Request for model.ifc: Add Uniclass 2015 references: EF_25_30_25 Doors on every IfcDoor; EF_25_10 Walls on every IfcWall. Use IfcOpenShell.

First a look at what the model holds.

```python
import ifcopenshell

model = ifcopenshell.open("model.ifc")
print(model.schema)
print("classifications:", [c.Name for c in model.by_type("IfcClassification")])
for ifc_class in ("IfcDoor", "IfcRoof", "IfcStair", "IfcWall", "IfcWindow"):
    print(ifc_class, len(model.by_type(ifc_class)))
```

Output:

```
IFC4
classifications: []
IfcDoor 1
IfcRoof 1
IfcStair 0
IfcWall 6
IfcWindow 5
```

```python
import ifcopenshell
import ifcopenshell.api.classification

model = ifcopenshell.open("model.ifc")

system = ifcopenshell.api.classification.add_classification(model, classification="Uniclass 2015")

codes = {
    "IfcDoor": ("EF_25_30_25", "Doors"),
    "IfcWall": ("EF_25_10", "Walls"),
}
for ifc_class, (code, name) in codes.items():
    products = model.by_type(ifc_class)
    ifcopenshell.api.classification.add_reference(
        model, products=products, classification=system, identification=code, name=name
    )
    print(code, len(products))

model.write("model_updated.ifc")
```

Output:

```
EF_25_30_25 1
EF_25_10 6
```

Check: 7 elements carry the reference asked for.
